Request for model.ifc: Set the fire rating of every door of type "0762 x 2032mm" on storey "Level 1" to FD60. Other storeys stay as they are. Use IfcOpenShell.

First a look at what the model holds.

```python
import ifcopenshell
import ifcopenshell.util.element

model = ifcopenshell.open("model.ifc")
print(model.schema)
storey = next(s for s in model.by_type("IfcBuildingStorey") if s.Name == "Level 1")
doors = [e for e in ifcopenshell.util.element.get_decomposition(storey) if e.is_a("IfcDoor")]
seen = {}
for e in doors:
    element_type = ifcopenshell.util.element.get_type(e)
    key = (element_type.Name if element_type != e and element_type else None, ifcopenshell.util.element.get_pset(e, "Pset_DoorCommon", "FireRating"))
    seen[key] = seen.get(key, 0) + 1
for (name, value), count in sorted(seen.items(), key=str):
    print(count, "x", name, "|", value)
```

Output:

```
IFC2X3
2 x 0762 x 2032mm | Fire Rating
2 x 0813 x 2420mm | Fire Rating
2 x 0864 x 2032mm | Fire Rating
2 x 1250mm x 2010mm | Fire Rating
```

```python
import ifcopenshell
import ifcopenshell.api.pset
import ifcopenshell.util.element

model = ifcopenshell.open("model.ifc")

storey = next(s for s in model.by_type("IfcBuildingStorey") if s.Name == "Level 1")
doors = [e for e in ifcopenshell.util.element.get_decomposition(storey) if e.is_a("IfcDoor")]

count = 0
for e in doors:
    element_type = ifcopenshell.util.element.get_type(e)
    if element_type in (None, e) or element_type.Name != "0762 x 2032mm":
        continue
    # add_pset returns the element's existing set when there is one.
    pset = ifcopenshell.api.pset.add_pset(model, product=e, name="Pset_DoorCommon")
    ifcopenshell.api.pset.edit_pset(model, pset=pset, properties={"FireRating": "FD60"})
    count += 1

print(count, "doors updated")

model.write("model_updated.ifc")
```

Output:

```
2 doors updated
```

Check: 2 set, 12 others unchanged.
